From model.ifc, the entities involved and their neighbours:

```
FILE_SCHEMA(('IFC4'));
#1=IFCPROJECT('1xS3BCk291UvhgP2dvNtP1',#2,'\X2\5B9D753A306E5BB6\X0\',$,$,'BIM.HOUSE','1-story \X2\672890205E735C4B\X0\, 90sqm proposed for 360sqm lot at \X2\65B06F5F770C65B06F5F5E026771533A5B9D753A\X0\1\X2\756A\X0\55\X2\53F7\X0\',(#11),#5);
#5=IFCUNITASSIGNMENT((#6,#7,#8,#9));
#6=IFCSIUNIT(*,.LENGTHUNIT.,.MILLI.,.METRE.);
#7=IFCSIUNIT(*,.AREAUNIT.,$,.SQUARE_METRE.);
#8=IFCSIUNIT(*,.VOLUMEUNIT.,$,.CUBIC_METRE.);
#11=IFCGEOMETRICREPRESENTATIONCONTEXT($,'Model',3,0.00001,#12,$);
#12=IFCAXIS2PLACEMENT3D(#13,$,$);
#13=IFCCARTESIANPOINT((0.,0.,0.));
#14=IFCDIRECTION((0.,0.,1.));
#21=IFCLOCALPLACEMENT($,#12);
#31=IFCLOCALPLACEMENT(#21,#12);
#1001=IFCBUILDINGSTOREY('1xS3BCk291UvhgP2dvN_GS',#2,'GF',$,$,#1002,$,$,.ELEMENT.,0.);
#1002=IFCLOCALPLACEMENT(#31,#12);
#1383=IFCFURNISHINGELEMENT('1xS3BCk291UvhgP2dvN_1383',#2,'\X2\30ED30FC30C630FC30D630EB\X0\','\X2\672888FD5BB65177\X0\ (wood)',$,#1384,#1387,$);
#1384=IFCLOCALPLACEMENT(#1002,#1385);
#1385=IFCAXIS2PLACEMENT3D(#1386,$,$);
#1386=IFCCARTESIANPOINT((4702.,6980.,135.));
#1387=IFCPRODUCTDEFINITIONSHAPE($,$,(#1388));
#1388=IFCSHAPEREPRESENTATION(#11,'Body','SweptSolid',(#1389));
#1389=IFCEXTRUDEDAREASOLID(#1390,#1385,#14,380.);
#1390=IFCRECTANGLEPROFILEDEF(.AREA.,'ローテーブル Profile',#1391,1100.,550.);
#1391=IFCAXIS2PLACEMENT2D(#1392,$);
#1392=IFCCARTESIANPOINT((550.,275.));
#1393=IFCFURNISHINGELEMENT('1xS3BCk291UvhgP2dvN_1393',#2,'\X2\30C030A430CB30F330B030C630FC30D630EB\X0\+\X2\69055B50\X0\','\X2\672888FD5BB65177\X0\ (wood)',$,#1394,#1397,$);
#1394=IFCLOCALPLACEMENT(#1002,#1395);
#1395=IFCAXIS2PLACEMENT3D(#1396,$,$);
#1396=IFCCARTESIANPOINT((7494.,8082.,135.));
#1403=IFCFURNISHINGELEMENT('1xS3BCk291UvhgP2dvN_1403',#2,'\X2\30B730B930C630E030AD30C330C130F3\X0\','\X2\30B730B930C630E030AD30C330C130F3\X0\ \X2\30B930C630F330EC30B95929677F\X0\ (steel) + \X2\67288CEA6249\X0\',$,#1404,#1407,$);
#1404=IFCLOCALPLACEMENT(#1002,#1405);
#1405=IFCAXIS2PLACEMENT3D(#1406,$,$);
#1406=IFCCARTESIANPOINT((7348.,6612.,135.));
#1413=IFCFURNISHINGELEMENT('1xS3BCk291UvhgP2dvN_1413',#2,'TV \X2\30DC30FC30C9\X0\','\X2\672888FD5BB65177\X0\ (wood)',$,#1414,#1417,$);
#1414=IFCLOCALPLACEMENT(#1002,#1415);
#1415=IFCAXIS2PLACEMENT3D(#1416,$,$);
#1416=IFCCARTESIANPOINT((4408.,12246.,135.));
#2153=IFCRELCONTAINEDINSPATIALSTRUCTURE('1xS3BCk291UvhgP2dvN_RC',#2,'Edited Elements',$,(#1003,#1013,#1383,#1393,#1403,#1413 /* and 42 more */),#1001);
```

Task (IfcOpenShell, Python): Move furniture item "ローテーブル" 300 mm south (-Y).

```python
import ifcopenshell
import ifcopenshell.api.geometry
import ifcopenshell.util.placement
import ifcopenshell.util.unit

model = ifcopenshell.open("model.ifc")
unit_scale = ifcopenshell.util.unit.calculate_unit_scale(model)

item = model.by_id(1383)
matrix = ifcopenshell.util.placement.get_local_placement(item.ObjectPlacement)
matrix[1, 3] -= 0.3 / unit_scale
ifcopenshell.api.geometry.edit_object_placement(model, product=item, matrix=matrix, is_si=False)

print(ifcopenshell.util.placement.get_local_placement(item.ObjectPlacement).round(3) + 0.0)

model.write("model_updated.ifc")
```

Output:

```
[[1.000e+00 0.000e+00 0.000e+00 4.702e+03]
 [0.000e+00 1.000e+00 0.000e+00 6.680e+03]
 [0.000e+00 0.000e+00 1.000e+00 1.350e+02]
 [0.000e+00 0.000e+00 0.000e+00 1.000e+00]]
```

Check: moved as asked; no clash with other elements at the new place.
